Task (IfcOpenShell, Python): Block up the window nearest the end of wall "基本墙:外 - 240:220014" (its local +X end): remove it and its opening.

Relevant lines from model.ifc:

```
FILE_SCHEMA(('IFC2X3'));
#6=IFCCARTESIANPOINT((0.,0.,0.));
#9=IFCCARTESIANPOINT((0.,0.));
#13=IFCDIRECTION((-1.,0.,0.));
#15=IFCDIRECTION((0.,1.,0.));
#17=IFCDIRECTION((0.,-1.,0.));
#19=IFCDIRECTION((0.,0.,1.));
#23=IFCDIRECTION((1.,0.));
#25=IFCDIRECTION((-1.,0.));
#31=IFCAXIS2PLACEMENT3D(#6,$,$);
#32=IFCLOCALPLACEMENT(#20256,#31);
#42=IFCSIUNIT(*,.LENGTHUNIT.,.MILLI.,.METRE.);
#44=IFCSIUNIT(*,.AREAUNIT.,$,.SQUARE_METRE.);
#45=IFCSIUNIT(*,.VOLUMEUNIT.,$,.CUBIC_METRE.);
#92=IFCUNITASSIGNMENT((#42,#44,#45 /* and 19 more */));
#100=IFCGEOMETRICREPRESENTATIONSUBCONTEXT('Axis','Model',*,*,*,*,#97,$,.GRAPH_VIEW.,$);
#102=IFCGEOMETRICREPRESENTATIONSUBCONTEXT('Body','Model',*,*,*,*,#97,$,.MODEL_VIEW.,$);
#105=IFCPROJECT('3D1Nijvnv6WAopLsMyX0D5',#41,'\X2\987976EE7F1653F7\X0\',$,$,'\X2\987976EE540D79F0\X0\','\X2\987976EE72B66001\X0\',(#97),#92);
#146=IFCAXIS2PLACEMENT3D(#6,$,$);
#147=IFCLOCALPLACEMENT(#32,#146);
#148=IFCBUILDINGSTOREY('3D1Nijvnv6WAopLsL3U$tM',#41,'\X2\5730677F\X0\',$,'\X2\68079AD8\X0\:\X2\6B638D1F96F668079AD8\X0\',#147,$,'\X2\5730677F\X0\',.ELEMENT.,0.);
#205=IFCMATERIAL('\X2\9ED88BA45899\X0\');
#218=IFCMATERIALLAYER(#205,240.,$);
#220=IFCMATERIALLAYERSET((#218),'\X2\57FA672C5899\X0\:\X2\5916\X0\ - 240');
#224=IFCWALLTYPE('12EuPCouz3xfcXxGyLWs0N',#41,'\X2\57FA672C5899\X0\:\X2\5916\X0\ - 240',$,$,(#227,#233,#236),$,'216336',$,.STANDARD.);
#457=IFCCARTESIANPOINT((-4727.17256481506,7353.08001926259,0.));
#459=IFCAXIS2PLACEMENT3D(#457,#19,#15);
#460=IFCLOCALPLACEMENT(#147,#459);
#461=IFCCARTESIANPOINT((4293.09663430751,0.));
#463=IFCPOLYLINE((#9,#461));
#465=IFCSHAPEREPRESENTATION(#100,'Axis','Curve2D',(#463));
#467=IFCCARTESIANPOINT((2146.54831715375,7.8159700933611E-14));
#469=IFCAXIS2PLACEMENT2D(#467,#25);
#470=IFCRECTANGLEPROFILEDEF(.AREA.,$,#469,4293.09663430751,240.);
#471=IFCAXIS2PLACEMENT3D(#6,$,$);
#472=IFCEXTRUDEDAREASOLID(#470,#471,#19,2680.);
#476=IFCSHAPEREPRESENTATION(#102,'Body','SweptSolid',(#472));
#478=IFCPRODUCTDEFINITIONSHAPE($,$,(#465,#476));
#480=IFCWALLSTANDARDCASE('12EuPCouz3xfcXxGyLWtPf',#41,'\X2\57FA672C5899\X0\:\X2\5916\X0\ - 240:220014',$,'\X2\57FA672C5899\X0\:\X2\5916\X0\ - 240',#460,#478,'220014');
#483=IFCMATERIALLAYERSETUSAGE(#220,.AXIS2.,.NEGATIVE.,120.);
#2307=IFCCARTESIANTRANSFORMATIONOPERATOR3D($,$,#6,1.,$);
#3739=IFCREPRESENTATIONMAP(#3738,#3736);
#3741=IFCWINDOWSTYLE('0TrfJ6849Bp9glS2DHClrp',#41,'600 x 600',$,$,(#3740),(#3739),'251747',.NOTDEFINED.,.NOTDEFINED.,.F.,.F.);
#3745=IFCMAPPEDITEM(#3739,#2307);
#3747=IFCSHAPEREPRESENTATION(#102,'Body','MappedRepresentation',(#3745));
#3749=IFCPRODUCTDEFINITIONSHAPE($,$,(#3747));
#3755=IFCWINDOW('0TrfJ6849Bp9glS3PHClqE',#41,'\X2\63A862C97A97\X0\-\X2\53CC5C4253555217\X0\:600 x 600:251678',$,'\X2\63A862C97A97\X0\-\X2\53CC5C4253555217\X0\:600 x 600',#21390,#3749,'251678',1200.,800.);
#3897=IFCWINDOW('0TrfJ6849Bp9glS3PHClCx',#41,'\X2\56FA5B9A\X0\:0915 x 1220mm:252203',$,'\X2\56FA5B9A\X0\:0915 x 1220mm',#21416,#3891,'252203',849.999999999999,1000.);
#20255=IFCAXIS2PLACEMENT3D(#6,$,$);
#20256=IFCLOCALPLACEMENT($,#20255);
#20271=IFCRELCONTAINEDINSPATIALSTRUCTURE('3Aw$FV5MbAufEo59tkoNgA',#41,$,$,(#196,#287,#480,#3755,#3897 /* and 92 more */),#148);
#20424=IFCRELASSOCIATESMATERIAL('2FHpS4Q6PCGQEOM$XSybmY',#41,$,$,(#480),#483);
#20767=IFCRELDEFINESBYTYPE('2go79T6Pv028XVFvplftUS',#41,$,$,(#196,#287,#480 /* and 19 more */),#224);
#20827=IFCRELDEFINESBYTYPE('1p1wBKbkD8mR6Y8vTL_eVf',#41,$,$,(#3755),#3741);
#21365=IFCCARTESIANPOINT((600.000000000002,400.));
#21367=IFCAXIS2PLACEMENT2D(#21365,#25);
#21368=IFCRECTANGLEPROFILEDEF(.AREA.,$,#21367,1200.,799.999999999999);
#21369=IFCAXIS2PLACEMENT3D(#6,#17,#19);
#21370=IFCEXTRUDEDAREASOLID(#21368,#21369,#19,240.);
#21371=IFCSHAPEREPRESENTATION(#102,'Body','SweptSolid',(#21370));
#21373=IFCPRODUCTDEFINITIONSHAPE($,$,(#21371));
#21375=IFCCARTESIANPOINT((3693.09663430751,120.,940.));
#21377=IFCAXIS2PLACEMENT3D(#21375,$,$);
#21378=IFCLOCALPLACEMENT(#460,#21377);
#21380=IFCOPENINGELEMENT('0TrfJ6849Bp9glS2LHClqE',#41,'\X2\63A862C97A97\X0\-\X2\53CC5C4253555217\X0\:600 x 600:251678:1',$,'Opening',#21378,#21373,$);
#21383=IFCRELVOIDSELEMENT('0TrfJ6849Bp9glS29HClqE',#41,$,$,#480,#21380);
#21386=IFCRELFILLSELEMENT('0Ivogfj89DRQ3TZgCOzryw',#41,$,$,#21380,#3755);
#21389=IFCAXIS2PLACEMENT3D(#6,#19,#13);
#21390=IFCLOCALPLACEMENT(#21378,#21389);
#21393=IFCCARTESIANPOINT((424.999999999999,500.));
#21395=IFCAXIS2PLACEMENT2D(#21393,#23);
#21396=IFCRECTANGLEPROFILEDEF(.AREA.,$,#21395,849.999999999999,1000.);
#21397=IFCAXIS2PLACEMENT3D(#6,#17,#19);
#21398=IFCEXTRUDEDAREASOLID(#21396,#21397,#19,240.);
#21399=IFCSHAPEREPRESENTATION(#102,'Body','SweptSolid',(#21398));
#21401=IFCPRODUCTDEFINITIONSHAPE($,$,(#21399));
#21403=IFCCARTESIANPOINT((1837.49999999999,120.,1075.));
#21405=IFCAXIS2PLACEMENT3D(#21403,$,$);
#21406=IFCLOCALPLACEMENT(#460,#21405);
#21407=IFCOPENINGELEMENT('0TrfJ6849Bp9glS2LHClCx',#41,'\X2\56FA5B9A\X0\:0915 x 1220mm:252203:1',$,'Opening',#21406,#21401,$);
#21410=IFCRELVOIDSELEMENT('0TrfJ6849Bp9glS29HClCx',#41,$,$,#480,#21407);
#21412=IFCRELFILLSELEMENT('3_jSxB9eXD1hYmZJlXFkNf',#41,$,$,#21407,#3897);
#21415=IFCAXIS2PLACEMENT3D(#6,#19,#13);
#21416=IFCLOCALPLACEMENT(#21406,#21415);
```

```python
import ifcopenshell
import ifcopenshell.api.feature
import ifcopenshell.api.root
import ifcopenshell.geom
import ifcopenshell.util.shape

model = ifcopenshell.open("model.ifc")
settings = ifcopenshell.geom.settings()


def volume(element):
    """Net volume in cubic metres, openings subtracted."""
    shape = ifcopenshell.geom.create_shape(settings, element)
    return ifcopenshell.util.shape.get_volume(shape.geometry)


window = model.by_id(3755)
opening = window.FillsVoids[0].RelatingOpeningElement
wall = opening.VoidsElements[0].RelatingBuildingElement
before = volume(wall)

ifcopenshell.api.root.remove_product(model, product=window)
ifcopenshell.api.feature.remove_feature(model, feature=opening)

after = volume(wall)

print(f"wall volume {before:.3f} -> {after:.3f} m3")

model.write("model_edited.ifc")
```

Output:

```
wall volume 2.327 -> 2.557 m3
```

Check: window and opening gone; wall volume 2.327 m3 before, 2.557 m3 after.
